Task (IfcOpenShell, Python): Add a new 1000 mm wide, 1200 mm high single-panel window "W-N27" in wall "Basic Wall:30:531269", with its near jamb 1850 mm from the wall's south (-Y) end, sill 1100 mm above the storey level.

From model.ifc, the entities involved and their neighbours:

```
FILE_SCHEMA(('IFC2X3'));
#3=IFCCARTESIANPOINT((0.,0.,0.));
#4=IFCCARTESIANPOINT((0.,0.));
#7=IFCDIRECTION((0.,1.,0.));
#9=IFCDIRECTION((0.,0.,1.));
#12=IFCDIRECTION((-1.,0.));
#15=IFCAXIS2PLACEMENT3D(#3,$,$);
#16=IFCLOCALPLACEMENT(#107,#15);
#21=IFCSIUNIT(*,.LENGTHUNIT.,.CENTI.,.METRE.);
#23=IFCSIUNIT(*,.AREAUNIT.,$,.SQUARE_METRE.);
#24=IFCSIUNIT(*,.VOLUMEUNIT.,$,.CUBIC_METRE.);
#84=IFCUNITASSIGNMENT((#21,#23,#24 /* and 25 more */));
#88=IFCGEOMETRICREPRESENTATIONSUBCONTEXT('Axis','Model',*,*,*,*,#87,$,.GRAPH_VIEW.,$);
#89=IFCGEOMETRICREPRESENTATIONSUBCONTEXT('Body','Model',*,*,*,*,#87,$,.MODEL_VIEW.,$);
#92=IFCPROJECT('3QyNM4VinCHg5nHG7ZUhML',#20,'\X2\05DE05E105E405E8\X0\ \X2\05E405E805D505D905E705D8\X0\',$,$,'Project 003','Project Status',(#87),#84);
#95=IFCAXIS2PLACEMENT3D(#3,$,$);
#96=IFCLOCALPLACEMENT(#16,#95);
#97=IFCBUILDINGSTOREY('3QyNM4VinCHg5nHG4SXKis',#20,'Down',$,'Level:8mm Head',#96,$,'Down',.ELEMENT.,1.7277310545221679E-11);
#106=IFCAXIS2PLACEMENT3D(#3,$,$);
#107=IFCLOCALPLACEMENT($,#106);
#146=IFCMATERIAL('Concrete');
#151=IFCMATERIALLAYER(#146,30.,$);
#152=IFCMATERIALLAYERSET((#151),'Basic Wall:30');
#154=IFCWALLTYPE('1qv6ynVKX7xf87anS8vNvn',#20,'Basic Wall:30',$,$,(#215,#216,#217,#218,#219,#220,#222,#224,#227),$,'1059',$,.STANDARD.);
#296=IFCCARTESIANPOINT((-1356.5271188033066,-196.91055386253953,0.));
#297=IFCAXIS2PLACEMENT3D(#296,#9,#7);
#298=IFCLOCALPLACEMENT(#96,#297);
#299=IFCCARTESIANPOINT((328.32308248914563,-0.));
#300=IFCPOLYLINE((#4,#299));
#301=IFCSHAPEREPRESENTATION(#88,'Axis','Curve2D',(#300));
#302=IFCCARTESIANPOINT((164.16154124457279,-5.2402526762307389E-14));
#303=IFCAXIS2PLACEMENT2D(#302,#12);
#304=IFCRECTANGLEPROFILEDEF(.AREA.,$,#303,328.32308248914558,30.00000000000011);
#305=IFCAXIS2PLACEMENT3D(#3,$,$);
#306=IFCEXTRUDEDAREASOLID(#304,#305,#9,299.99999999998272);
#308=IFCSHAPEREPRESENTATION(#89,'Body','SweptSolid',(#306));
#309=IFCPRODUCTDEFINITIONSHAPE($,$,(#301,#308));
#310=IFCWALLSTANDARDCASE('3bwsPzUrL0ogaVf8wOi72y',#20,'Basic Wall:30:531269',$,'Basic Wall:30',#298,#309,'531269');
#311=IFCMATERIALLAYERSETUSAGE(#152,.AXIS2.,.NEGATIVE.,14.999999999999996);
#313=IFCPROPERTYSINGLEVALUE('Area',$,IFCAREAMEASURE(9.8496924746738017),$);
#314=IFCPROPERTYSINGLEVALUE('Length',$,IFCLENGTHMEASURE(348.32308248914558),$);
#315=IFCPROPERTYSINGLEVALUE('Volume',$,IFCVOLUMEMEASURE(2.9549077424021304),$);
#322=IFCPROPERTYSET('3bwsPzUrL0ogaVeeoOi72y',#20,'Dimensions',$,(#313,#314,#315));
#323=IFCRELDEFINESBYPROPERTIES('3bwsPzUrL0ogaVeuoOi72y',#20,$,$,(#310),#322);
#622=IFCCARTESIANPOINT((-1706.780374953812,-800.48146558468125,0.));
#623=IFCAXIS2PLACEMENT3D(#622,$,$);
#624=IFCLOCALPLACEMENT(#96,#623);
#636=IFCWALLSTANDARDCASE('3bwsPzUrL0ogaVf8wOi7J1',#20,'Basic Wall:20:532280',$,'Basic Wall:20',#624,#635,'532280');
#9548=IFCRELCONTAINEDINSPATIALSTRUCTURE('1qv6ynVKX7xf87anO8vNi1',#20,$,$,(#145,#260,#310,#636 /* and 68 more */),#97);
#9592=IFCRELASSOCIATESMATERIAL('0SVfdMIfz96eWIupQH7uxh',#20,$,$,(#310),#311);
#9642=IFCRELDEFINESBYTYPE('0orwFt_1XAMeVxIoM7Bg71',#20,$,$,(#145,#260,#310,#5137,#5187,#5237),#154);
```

```python
import numpy as np
import ifcopenshell
import ifcopenshell.api.feature
import ifcopenshell.api.geometry
import ifcopenshell.api.pset
import ifcopenshell.api.root
import ifcopenshell.api.spatial
import ifcopenshell.api.type
import ifcopenshell.geom
import ifcopenshell.util.element
import ifcopenshell.util.placement
import ifcopenshell.util.representation
import ifcopenshell.util.shape
import ifcopenshell.util.unit

model = ifcopenshell.open("model.ifc")
unit_scale = ifcopenshell.util.unit.calculate_unit_scale(model)
area_scale = ifcopenshell.util.unit.calculate_unit_scale(model, "AREAUNIT")
volume_scale = ifcopenshell.util.unit.calculate_unit_scale(model, "VOLUMEUNIT")
settings = ifcopenshell.geom.settings()


def volume(element):
    """Net volume in cubic metres, openings subtracted."""
    shape = ifcopenshell.geom.create_shape(settings, element)
    return ifcopenshell.util.shape.get_volume(shape.geometry)


wall = model.by_guid("3bwsPzUrL0ogaVf8wOi72y")
storey = ifcopenshell.util.element.get_container(wall, ifc_class="IfcBuildingStorey")
context = ifcopenshell.util.representation.get_context(model, "Model", "Body", "MODEL_VIEW")
before = volume(wall)

width, height, from_end, sill = 1, 1.2, 1.85, 1.1  # metres

# The wall runs along its own X axis, and the end named is its -X end.
wall_shape = ifcopenshell.geom.create_shape(settings, wall)
x, y, z = ifcopenshell.util.shape.get_vertices(wall_shape.geometry).T
start = x.min() + from_end
face, thickness = float(y.min()), float(y.max() - y.min())
wall_matrix = ifcopenshell.util.placement.get_local_placement(wall.ObjectPlacement)
level = ifcopenshell.util.placement.get_local_placement(storey.ObjectPlacement)[2, 3]


def in_wall(x, y):
    """Placement at x, y metres in the wall's axes, at sill height."""
    matrix = wall_matrix.copy()
    matrix[:, 3] = wall_matrix @ np.array([x / unit_scale, y / unit_scale, 0.0, 1.0])
    matrix[2, 3] = level + sill / unit_scale
    return matrix


# Opening: a box that overshoots both wall faces by 50 mm.
opening = ifcopenshell.api.root.create_entity(model, ifc_class="IfcOpeningElement")
box = ifcopenshell.api.geometry.add_wall_representation(
    model, context=context, length=width, height=height, thickness=thickness + 0.1
)
ifcopenshell.api.geometry.assign_representation(model, product=opening, representation=box)
ifcopenshell.api.geometry.edit_object_placement(model, product=opening, matrix=in_wall(start, face - 0.05), is_si=False)
ifcopenshell.api.feature.add_feature(model, feature=opening, element=wall)

window = ifcopenshell.api.root.create_entity(model, ifc_class="IfcWindow", name="W-N27")
window.OverallWidth, window.OverallHeight = width / unit_scale, height / unit_scale
body = ifcopenshell.api.geometry.add_window_representation(
    model,
    context=context,
    overall_width=window.OverallWidth,
    overall_height=window.OverallHeight,
    partition_type="SINGLE_PANEL",
)
ifcopenshell.api.geometry.assign_representation(model, product=window, representation=body)
ifcopenshell.api.spatial.assign_container(model, products=[window], relating_structure=storey)
fills = ifcopenshell.api.feature.add_filling(model, opening=opening, element=window)
fills.OwnerHistory = window.OwnerHistory  # required in IFC2X3

# IFC2X3 keeps the operation on the window style.
style = ifcopenshell.api.root.create_entity(model, ifc_class="IfcWindowStyle", name="W-N27")
style.OperationType, style.ConstructionType = "SINGLE_PANEL", "NOTDEFINED"
style.ParameterTakesPrecedence = style.Sizeable = False
ifcopenshell.api.type.assign_type(model, related_objects=[window], relating_type=style)

# Centre the window in the wall's thickness.
ifcopenshell.api.geometry.edit_object_placement(model, product=window, matrix=in_wall(start, face), is_si=False)
window_shape = ifcopenshell.geom.create_shape(settings, window)
depth = ifcopenshell.util.shape.get_vertices(window_shape.geometry)[:, 1]
offset = face + thickness / 2 - (depth.min() + depth.max()) / 2
ifcopenshell.api.geometry.edit_object_placement(model, product=window, matrix=in_wall(start, offset), is_si=False)

after = volume(wall)

# Update the wall's stored quantities.
pset = model.by_id(ifcopenshell.util.element.get_pset(wall, "Dimensions", should_inherit=False)["id"])
ifcopenshell.api.pset.edit_pset(model, pset=pset, properties={
    "Area": model.create_entity("IfcAreaMeasure", after / thickness / area_scale),
    "Volume": model.create_entity("IfcVolumeMeasure", after / volume_scale),
})

print(f"wall volume {before:.3f} -> {after:.3f} m3")

model.write("model_v2.ifc")
```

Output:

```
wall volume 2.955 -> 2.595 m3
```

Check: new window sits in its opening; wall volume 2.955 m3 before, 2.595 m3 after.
